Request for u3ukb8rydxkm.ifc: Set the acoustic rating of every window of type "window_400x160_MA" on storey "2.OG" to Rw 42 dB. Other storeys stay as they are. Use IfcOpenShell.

First a look at what the model holds.

```python
import ifcopenshell
import ifcopenshell.util.element

model = ifcopenshell.open("u3ukb8rydxkm.ifc")
print(model.schema)
storey = next(s for s in model.by_type("IfcBuildingStorey") if s.Name == "2.OG")
windows = [e for e in ifcopenshell.util.element.get_decomposition(storey) if e.is_a("IfcWindow")]
seen = {}
for e in windows:
    element_type = ifcopenshell.util.element.get_type(e)
    key = (element_type.Name if element_type != e and element_type else None, ifcopenshell.util.element.get_pset(e, "Pset_WindowCommon", "AcousticRating"))
    seen[key] = seen.get(key, 0) + 1
for (name, value), count in sorted(seen.items(), key=str):
    print(count, "x", name, "|", value)
```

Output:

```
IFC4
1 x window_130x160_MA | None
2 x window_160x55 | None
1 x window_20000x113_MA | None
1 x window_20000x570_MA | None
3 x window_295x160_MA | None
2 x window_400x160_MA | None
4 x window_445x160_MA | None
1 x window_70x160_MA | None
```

```python
import ifcopenshell
import ifcopenshell.api.pset
import ifcopenshell.util.element

model = ifcopenshell.open("u3ukb8rydxkm.ifc")

storey = next(s for s in model.by_type("IfcBuildingStorey") if s.Name == "2.OG")
windows = [e for e in ifcopenshell.util.element.get_decomposition(storey) if e.is_a("IfcWindow")]

count = 0
for e in windows:
    element_type = ifcopenshell.util.element.get_type(e)
    if element_type in (None, e) or element_type.Name != "window_400x160_MA":
        continue
    # add_pset returns the element's existing set when there is one.
    pset = ifcopenshell.api.pset.add_pset(model, product=e, name="Pset_WindowCommon")
    ifcopenshell.api.pset.edit_pset(model, pset=pset, properties={"AcousticRating": "Rw 42 dB"})
    count += 1

print(count, "windows updated")

model.write("u3ukb8rydxkm_updated.ifc")
```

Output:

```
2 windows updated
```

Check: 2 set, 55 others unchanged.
